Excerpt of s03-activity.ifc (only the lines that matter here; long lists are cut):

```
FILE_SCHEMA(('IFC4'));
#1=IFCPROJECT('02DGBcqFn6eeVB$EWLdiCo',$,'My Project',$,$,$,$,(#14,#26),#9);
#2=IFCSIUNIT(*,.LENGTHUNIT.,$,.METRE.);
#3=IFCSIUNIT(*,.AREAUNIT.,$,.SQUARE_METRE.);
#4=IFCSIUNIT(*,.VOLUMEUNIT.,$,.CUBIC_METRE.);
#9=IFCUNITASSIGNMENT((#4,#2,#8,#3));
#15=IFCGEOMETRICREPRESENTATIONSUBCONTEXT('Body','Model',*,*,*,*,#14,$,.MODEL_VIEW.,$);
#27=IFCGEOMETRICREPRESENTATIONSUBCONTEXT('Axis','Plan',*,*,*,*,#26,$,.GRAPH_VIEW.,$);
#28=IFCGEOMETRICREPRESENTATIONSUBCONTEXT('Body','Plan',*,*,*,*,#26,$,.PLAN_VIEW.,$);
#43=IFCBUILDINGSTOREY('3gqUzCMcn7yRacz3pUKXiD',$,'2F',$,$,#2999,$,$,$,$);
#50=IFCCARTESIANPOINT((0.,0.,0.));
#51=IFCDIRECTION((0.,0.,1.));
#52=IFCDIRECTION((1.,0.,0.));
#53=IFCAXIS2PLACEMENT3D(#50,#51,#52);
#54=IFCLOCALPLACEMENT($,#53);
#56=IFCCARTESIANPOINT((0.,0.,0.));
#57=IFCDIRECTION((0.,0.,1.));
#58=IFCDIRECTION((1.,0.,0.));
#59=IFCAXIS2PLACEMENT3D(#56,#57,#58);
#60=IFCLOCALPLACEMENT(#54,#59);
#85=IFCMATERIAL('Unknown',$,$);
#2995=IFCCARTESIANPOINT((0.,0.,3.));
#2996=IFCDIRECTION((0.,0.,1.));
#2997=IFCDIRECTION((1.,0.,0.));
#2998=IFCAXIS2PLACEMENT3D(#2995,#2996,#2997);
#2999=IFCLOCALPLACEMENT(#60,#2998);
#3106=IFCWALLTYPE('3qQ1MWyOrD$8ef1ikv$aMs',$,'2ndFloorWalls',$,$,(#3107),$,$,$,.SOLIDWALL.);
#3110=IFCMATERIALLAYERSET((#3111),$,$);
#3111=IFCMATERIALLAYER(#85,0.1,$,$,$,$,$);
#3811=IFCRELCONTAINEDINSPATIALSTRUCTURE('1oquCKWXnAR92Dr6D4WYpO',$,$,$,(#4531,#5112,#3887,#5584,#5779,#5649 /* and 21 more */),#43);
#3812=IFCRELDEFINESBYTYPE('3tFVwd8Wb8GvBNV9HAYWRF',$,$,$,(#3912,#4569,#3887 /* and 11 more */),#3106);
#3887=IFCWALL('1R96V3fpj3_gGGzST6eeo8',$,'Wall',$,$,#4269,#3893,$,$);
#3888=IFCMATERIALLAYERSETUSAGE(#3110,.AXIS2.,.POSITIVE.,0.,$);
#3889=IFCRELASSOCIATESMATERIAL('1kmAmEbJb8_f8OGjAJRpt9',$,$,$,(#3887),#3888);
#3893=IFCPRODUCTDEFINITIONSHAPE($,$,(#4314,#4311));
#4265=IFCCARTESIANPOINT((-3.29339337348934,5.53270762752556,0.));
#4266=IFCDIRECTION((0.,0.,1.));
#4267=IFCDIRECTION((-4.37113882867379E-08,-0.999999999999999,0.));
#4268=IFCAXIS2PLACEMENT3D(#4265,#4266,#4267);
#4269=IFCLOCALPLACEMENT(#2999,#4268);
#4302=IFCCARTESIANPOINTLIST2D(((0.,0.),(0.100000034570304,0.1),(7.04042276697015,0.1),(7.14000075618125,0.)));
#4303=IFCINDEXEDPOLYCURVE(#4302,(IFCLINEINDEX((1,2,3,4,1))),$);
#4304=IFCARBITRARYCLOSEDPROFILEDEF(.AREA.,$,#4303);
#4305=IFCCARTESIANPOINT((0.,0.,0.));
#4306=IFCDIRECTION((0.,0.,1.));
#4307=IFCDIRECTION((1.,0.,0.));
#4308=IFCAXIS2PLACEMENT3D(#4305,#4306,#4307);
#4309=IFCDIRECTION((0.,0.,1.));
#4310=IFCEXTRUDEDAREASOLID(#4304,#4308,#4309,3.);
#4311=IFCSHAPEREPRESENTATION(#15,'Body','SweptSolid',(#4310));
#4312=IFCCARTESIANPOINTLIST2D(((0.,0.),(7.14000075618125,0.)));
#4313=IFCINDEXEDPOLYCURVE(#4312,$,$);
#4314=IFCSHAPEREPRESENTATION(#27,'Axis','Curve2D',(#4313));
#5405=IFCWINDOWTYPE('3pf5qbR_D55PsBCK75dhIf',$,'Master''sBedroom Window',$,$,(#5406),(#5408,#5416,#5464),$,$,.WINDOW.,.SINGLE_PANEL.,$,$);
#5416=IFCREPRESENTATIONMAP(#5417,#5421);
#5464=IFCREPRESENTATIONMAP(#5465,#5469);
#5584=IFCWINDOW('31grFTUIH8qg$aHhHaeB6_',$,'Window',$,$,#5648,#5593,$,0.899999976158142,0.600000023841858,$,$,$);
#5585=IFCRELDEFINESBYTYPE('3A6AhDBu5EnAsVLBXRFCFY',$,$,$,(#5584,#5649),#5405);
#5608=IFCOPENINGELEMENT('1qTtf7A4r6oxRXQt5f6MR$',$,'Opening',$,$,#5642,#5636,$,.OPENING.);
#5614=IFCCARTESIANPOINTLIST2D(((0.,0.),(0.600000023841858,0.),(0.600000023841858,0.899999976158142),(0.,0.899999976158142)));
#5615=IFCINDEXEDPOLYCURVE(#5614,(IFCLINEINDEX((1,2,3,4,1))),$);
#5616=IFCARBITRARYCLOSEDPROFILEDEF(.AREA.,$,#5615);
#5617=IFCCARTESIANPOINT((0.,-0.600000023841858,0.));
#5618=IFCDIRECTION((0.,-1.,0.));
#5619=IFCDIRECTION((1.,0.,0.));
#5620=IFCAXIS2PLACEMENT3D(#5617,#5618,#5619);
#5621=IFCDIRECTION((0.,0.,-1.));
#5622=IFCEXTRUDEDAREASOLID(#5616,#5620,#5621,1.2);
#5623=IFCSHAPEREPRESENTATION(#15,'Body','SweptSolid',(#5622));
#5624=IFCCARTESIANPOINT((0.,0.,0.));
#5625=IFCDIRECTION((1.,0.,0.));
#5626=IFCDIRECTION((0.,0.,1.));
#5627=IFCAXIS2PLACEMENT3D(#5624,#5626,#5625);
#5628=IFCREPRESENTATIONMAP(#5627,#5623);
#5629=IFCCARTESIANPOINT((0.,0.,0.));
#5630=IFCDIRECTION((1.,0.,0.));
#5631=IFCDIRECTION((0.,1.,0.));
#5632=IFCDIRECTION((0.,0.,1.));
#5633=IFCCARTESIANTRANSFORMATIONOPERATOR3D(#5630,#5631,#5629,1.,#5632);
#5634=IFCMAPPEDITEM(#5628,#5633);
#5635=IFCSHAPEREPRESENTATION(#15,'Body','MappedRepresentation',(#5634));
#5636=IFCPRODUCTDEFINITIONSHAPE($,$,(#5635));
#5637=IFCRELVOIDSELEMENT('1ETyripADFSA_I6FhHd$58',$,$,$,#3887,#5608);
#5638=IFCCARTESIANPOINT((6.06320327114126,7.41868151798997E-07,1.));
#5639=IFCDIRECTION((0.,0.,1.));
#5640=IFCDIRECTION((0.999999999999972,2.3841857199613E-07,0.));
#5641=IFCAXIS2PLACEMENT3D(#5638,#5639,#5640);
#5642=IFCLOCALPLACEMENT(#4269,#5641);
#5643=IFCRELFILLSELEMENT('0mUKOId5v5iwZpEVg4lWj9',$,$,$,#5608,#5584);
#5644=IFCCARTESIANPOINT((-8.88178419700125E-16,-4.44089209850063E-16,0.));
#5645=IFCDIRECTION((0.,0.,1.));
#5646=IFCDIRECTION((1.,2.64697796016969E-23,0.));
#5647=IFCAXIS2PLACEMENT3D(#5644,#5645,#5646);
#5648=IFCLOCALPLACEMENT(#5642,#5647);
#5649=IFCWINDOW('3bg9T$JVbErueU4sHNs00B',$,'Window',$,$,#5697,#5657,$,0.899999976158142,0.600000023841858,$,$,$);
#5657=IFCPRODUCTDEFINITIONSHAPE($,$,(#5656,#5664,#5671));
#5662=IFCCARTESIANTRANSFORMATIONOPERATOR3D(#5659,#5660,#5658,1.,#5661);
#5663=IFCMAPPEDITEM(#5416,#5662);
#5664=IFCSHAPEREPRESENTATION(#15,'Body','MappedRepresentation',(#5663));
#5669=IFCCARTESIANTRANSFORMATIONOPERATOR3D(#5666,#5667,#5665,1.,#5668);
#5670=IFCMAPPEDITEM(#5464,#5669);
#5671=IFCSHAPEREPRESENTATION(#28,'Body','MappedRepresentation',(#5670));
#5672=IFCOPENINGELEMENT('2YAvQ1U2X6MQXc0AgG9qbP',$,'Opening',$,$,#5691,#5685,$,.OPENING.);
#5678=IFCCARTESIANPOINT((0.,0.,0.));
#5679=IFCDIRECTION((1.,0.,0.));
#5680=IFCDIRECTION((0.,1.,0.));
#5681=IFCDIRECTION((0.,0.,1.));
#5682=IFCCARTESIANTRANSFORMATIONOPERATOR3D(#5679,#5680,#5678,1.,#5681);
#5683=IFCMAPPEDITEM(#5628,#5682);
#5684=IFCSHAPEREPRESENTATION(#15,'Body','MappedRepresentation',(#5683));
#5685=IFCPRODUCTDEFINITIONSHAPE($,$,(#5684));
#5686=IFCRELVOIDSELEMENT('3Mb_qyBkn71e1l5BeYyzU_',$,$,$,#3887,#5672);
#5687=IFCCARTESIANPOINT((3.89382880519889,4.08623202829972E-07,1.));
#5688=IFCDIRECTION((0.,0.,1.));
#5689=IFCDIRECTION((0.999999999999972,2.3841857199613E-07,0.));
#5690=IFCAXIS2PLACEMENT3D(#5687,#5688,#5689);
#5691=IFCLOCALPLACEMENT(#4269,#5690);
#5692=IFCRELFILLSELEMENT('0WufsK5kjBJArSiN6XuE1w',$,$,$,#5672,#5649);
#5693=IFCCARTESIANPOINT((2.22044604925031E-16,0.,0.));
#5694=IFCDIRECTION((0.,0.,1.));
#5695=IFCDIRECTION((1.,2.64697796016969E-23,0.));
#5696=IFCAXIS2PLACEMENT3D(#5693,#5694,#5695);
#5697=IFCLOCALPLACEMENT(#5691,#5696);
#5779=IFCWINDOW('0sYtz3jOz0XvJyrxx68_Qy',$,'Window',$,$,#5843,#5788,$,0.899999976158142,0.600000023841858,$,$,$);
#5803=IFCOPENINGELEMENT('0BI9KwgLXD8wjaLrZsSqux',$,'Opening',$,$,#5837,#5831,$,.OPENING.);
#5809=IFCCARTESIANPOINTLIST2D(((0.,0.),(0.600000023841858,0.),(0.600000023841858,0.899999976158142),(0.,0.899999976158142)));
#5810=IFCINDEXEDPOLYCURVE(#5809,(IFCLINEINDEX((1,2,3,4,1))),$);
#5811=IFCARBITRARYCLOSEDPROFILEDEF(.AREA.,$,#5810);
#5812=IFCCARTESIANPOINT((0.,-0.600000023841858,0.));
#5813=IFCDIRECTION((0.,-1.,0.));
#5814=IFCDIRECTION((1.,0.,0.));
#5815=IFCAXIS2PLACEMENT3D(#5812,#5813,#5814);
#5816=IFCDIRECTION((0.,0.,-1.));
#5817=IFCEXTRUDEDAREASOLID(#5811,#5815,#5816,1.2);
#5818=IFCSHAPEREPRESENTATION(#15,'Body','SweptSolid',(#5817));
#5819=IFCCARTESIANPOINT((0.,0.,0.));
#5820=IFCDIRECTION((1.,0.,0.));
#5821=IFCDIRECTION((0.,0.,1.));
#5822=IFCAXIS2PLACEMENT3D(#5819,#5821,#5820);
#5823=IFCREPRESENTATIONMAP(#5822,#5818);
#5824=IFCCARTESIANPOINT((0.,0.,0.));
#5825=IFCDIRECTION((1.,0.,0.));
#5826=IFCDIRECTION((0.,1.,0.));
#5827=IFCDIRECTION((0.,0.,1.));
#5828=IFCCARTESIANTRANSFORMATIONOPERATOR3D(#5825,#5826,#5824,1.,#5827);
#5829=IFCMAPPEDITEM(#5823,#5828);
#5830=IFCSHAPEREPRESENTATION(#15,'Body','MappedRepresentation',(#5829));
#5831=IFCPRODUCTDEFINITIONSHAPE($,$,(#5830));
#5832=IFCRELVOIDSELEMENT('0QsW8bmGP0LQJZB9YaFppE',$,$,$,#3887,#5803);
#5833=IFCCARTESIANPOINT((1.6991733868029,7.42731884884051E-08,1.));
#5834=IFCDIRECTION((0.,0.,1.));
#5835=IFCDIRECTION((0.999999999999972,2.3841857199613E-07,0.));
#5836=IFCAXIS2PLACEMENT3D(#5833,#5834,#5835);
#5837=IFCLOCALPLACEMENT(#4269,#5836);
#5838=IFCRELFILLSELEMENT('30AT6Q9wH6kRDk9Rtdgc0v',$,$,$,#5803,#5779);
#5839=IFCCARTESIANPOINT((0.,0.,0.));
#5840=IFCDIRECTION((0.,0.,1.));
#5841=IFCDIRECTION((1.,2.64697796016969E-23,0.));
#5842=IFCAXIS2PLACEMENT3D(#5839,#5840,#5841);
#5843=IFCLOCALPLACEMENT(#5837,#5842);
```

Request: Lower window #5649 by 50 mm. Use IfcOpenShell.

```python
import numpy as np
import ifcopenshell
import ifcopenshell.api.geometry
import ifcopenshell.util.placement
import ifcopenshell.util.unit

model = ifcopenshell.open("s03-activity.ifc")
unit_scale = ifcopenshell.util.unit.calculate_unit_scale(model)

window = model.by_id(5649)
opening = window.FillsVoids[0].RelatingOpeningElement
dz = -0.05 / unit_scale

shift = np.array([0.0, 0.0, dz])
# The window is placed relative to its opening, so it follows when the opening moves.
matrix = ifcopenshell.util.placement.get_local_placement(opening.ObjectPlacement)
matrix[:3, 3] += shift
ifcopenshell.api.geometry.edit_object_placement(
    model, product=opening, matrix=matrix, is_si=False, should_transform_children=True
)

print(f"moved by {dz * unit_scale:+.3f} m")

model.write("s03-activity-out.ifc")
```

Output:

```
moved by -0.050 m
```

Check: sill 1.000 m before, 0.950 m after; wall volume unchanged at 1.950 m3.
